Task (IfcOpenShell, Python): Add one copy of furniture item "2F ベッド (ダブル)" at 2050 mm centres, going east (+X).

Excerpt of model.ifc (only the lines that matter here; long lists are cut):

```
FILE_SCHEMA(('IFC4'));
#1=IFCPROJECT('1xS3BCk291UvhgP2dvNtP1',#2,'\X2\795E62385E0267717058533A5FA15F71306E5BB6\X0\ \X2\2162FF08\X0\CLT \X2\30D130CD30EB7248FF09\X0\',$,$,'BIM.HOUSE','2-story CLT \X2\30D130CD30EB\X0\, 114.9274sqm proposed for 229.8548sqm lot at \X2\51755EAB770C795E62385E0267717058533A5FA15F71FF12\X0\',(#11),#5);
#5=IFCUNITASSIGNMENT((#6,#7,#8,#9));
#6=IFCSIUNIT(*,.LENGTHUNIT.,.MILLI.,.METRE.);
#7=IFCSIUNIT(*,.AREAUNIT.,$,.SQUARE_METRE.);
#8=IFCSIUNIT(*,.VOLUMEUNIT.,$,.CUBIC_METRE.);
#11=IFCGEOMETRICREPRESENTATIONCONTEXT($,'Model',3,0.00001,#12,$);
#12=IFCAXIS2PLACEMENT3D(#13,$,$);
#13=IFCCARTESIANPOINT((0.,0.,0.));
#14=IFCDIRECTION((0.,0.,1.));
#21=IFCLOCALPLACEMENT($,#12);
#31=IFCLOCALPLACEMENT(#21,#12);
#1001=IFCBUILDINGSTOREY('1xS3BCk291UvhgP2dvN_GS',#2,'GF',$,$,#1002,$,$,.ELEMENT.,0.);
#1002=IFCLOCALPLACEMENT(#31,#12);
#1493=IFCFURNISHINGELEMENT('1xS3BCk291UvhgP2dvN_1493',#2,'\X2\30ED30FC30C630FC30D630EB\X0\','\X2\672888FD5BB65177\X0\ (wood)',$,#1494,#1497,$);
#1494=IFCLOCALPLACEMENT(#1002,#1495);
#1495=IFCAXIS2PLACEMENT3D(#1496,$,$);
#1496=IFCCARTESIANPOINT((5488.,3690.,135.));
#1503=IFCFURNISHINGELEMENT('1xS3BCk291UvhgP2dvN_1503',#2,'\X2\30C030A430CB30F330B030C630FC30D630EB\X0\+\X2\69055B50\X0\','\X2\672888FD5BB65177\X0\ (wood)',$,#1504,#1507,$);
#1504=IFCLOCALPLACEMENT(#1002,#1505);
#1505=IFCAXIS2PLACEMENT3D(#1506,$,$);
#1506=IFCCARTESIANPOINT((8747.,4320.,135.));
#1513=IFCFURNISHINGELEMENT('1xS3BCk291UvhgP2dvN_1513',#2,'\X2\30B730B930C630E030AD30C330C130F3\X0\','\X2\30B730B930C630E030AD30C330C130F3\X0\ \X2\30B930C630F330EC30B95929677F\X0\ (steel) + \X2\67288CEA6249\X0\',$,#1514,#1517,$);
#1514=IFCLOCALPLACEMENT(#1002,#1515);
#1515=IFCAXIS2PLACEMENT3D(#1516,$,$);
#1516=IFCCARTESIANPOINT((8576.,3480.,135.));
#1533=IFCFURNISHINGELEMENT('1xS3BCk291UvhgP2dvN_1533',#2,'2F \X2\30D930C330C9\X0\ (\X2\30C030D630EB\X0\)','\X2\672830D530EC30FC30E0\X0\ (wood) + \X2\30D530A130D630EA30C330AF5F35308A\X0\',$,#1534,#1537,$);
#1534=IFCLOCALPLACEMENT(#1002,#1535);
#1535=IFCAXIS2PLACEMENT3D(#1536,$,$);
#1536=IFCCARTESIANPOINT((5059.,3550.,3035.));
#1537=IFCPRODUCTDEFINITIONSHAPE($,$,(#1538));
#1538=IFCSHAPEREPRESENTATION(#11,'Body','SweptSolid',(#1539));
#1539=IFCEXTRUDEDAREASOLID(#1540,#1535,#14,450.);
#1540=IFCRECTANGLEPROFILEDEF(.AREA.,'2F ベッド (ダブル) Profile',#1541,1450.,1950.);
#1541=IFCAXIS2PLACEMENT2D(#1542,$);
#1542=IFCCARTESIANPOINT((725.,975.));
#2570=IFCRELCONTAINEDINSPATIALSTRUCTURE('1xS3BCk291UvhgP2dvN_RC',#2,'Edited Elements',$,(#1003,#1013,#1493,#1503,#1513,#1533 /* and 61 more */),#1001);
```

```python
import numpy as np
import ifcopenshell
import ifcopenshell.api.geometry
import ifcopenshell.api.root
import ifcopenshell.util.element
import ifcopenshell.util.placement
import ifcopenshell.util.unit

model = ifcopenshell.open("model.ifc")
unit_scale = ifcopenshell.util.unit.calculate_unit_scale(model)


def reuse_history(source, copy):
    """copy_class also copies each property set's owner history, people and application; keep the originals."""
    for rel in copy.IsDefinedBy:
        if rel.is_a("IfcRelDefinesByProperties") and (history := rel.RelatingPropertyDefinition.OwnerHistory):
            rel.RelatingPropertyDefinition.OwnerHistory = source.OwnerHistory
            ifcopenshell.util.element.remove_deep2(model, history)


source = model.by_guid("1xS3BCk291UvhgP2dvN_1533")
base = ifcopenshell.util.placement.get_local_placement(source.ObjectPlacement)
step = np.array([1.0, 0.0, 0.0]) * 2.05 / unit_scale

for i in range(1, 2):
    copy = ifcopenshell.api.root.copy_class(model, product=source)
    copy.Representation = ifcopenshell.util.element.copy_deep(
        model, source.Representation, exclude=["IfcGeometricRepresentationContext", "IfcRepresentationMap"]
    )
    reuse_history(source, copy)
    matrix = base.copy()
    matrix[:3, 3] += i * step
    print("added at", matrix[:3, 3].round(3) + 0.0)
    ifcopenshell.api.geometry.edit_object_placement(model, product=copy, matrix=matrix, is_si=False)

model.write("model_updated.ifc")
```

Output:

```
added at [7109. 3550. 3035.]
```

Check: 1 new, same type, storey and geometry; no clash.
